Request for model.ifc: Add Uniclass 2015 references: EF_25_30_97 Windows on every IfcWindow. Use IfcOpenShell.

First a look at what the model holds.

```python
import ifcopenshell

model = ifcopenshell.open("model.ifc")
print(model.schema)
print("classifications:", [c.Name for c in model.by_type("IfcClassification")])
for ifc_class in ("IfcDoor", "IfcRoof", "IfcStair", "IfcWall", "IfcWindow"):
    print(ifc_class, len(model.by_type(ifc_class)))
```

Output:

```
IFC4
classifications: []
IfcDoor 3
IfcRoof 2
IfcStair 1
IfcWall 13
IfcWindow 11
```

```python
import ifcopenshell
import ifcopenshell.api.classification

model = ifcopenshell.open("model.ifc")

system = ifcopenshell.api.classification.add_classification(model, classification="Uniclass 2015")

codes = {
    "IfcWindow": ("EF_25_30_97", "Windows"),
}
for ifc_class, (code, name) in codes.items():
    products = model.by_type(ifc_class)
    ifcopenshell.api.classification.add_reference(
        model, products=products, classification=system, identification=code, name=name
    )
    print(code, len(products))

model.write("model-out.ifc")
```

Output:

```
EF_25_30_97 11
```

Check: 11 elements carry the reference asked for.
